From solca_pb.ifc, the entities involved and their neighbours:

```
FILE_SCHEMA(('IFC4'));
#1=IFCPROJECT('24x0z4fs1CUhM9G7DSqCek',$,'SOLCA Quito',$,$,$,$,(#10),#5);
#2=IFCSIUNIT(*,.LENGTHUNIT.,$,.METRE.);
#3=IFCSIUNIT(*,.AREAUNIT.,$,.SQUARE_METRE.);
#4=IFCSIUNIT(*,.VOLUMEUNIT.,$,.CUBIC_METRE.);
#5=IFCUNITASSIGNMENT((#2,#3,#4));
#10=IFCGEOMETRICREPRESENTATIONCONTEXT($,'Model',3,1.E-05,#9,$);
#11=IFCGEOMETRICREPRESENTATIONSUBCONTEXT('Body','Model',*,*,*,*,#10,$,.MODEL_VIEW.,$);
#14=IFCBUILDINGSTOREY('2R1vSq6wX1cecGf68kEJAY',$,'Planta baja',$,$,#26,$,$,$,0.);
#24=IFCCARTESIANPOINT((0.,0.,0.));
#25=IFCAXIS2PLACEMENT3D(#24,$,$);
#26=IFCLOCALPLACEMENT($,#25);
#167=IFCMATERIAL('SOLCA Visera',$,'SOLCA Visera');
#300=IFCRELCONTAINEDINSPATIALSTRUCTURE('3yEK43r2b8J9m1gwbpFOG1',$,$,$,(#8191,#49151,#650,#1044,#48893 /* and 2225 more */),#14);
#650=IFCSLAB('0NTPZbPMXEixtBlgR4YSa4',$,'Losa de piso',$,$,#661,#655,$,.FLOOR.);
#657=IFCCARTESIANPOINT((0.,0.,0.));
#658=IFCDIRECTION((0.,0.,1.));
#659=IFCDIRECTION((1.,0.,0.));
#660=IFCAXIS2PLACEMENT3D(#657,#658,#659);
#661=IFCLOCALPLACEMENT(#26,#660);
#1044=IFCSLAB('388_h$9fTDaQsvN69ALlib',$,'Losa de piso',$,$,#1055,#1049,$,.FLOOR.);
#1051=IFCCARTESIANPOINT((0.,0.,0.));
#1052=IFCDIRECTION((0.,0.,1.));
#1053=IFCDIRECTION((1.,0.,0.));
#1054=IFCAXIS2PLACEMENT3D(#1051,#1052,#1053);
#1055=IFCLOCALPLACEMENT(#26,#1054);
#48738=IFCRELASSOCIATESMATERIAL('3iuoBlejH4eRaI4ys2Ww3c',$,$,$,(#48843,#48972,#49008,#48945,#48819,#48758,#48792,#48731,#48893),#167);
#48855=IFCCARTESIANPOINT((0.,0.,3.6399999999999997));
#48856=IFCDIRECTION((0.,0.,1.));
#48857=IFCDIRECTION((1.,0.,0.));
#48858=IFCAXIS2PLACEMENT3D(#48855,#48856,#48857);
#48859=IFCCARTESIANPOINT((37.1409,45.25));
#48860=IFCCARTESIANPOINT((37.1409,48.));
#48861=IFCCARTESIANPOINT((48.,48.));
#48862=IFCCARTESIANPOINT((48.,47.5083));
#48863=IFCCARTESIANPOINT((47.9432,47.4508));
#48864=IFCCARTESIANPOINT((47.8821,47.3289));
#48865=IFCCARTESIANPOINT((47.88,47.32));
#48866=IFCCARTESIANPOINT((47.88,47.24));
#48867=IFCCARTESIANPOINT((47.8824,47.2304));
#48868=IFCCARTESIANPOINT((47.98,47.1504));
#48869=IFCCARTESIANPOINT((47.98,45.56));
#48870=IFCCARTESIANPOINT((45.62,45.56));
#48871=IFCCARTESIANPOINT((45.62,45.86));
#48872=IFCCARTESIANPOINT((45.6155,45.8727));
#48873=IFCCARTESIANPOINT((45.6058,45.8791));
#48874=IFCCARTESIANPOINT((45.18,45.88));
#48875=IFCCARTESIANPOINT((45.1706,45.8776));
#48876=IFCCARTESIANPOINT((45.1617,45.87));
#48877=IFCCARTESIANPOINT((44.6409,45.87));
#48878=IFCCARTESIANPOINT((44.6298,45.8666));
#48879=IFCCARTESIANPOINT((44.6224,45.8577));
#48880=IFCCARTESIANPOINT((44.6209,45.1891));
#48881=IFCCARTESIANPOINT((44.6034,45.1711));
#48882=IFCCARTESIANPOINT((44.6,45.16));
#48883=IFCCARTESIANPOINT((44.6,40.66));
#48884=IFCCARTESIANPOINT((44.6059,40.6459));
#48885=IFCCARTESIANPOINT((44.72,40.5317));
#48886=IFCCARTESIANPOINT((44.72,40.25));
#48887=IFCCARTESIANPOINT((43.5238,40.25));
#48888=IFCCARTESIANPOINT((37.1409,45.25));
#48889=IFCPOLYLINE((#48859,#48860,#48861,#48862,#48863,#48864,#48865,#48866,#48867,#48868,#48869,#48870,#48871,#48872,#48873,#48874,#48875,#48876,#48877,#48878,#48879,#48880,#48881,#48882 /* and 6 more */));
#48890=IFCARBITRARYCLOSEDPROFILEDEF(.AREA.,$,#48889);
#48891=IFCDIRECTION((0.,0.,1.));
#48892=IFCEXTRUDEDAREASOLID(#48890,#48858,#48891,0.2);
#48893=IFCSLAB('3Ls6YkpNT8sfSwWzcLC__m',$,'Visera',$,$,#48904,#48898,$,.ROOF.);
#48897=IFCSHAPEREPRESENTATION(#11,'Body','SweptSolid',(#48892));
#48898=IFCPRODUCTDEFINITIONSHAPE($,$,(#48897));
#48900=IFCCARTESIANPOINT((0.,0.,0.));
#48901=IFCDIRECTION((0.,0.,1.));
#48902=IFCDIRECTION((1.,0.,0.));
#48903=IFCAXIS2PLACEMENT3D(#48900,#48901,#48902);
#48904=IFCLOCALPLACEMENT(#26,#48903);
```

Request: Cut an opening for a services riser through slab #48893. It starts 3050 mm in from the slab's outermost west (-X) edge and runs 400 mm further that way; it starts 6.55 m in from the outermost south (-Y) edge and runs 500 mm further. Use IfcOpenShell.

```python
import numpy as np
import ifcopenshell
import ifcopenshell.api.feature
import ifcopenshell.api.geometry
import ifcopenshell.api.root
import ifcopenshell.geom
import ifcopenshell.util.placement
import ifcopenshell.util.representation
import ifcopenshell.util.shape
import ifcopenshell.util.unit

model = ifcopenshell.open("solca_pb.ifc")
unit_scale = ifcopenshell.util.unit.calculate_unit_scale(model)
settings = ifcopenshell.geom.settings()


def volume(element):
    """Net volume in cubic metres, openings subtracted."""
    shape = ifcopenshell.geom.create_shape(settings, element)
    return ifcopenshell.util.shape.get_volume(shape.geometry)


slab = model.by_guid("3Ls6YkpNT8sfSwWzcLC__m")
before = volume(slab)

# Extent in the slab's own axes, in metres. The edges named are its -X and -Y sides.
slab_shape = ifcopenshell.geom.create_shape(settings, slab)
vertices = ifcopenshell.util.shape.get_vertices(slab_shape.geometry)
x_min, y_min, bottom = vertices.min(axis=0)
top = vertices[:, 2].max()

opening = ifcopenshell.api.root.create_entity(model, ifc_class="IfcOpeningElement", name="Services riser opening", predefined_type="OPENING")
context = ifcopenshell.util.representation.get_context(model, "Model", "Body", "MODEL_VIEW")
width, depth = 0.4, 0.5
outline = [(0.0, 0.0), (width, 0.0), (width, depth), (0.0, depth), (0.0, 0.0)]
# Overshoot both faces by 50 mm so the cut is clean.
shape = ifcopenshell.api.geometry.add_slab_representation(
    model, context=context, depth=top - bottom + 0.1, polyline=outline
)
ifcopenshell.api.geometry.assign_representation(model, product=opening, representation=shape)

matrix = ifcopenshell.util.placement.get_local_placement(slab.ObjectPlacement)
matrix[:, 3] = matrix @ np.append(np.array([x_min + 3.05, y_min + 6.55, bottom - 0.05]) / unit_scale, 1.0)
ifcopenshell.api.geometry.edit_object_placement(model, product=opening, matrix=matrix, is_si=False)
ifcopenshell.api.feature.add_feature(model, feature=opening, element=slab)

after = volume(slab)

print(f"slab volume {before:.3f} -> {after:.3f} m3")

model.write("solca_pb_updated.ifc")
```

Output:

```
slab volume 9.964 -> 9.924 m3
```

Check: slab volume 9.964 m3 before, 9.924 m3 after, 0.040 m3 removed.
